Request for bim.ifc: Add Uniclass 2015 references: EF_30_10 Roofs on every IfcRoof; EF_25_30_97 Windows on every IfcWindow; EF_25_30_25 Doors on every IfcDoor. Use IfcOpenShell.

First a look at what the model holds.

```python
import ifcopenshell

model = ifcopenshell.open("bim.ifc")
print(model.schema)
print("classifications:", [c.Name for c in model.by_type("IfcClassification")])
for ifc_class in ("IfcDoor", "IfcRoof", "IfcStair", "IfcWall", "IfcWindow"):
    print(ifc_class, len(model.by_type(ifc_class)))
```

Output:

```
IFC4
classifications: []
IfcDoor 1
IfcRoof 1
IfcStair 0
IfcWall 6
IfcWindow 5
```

```python
import ifcopenshell
import ifcopenshell.api.classification

model = ifcopenshell.open("bim.ifc")

system = ifcopenshell.api.classification.add_classification(model, classification="Uniclass 2015")

codes = {
    "IfcRoof": ("EF_30_10", "Roofs"),
    "IfcWindow": ("EF_25_30_97", "Windows"),
    "IfcDoor": ("EF_25_30_25", "Doors"),
}
for ifc_class, (code, name) in codes.items():
    products = model.by_type(ifc_class)
    ifcopenshell.api.classification.add_reference(
        model, products=products, classification=system, identification=code, name=name
    )
    print(code, len(products))

model.write("bim_edited.ifc")
```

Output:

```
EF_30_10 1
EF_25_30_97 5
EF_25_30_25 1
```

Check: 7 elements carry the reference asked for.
